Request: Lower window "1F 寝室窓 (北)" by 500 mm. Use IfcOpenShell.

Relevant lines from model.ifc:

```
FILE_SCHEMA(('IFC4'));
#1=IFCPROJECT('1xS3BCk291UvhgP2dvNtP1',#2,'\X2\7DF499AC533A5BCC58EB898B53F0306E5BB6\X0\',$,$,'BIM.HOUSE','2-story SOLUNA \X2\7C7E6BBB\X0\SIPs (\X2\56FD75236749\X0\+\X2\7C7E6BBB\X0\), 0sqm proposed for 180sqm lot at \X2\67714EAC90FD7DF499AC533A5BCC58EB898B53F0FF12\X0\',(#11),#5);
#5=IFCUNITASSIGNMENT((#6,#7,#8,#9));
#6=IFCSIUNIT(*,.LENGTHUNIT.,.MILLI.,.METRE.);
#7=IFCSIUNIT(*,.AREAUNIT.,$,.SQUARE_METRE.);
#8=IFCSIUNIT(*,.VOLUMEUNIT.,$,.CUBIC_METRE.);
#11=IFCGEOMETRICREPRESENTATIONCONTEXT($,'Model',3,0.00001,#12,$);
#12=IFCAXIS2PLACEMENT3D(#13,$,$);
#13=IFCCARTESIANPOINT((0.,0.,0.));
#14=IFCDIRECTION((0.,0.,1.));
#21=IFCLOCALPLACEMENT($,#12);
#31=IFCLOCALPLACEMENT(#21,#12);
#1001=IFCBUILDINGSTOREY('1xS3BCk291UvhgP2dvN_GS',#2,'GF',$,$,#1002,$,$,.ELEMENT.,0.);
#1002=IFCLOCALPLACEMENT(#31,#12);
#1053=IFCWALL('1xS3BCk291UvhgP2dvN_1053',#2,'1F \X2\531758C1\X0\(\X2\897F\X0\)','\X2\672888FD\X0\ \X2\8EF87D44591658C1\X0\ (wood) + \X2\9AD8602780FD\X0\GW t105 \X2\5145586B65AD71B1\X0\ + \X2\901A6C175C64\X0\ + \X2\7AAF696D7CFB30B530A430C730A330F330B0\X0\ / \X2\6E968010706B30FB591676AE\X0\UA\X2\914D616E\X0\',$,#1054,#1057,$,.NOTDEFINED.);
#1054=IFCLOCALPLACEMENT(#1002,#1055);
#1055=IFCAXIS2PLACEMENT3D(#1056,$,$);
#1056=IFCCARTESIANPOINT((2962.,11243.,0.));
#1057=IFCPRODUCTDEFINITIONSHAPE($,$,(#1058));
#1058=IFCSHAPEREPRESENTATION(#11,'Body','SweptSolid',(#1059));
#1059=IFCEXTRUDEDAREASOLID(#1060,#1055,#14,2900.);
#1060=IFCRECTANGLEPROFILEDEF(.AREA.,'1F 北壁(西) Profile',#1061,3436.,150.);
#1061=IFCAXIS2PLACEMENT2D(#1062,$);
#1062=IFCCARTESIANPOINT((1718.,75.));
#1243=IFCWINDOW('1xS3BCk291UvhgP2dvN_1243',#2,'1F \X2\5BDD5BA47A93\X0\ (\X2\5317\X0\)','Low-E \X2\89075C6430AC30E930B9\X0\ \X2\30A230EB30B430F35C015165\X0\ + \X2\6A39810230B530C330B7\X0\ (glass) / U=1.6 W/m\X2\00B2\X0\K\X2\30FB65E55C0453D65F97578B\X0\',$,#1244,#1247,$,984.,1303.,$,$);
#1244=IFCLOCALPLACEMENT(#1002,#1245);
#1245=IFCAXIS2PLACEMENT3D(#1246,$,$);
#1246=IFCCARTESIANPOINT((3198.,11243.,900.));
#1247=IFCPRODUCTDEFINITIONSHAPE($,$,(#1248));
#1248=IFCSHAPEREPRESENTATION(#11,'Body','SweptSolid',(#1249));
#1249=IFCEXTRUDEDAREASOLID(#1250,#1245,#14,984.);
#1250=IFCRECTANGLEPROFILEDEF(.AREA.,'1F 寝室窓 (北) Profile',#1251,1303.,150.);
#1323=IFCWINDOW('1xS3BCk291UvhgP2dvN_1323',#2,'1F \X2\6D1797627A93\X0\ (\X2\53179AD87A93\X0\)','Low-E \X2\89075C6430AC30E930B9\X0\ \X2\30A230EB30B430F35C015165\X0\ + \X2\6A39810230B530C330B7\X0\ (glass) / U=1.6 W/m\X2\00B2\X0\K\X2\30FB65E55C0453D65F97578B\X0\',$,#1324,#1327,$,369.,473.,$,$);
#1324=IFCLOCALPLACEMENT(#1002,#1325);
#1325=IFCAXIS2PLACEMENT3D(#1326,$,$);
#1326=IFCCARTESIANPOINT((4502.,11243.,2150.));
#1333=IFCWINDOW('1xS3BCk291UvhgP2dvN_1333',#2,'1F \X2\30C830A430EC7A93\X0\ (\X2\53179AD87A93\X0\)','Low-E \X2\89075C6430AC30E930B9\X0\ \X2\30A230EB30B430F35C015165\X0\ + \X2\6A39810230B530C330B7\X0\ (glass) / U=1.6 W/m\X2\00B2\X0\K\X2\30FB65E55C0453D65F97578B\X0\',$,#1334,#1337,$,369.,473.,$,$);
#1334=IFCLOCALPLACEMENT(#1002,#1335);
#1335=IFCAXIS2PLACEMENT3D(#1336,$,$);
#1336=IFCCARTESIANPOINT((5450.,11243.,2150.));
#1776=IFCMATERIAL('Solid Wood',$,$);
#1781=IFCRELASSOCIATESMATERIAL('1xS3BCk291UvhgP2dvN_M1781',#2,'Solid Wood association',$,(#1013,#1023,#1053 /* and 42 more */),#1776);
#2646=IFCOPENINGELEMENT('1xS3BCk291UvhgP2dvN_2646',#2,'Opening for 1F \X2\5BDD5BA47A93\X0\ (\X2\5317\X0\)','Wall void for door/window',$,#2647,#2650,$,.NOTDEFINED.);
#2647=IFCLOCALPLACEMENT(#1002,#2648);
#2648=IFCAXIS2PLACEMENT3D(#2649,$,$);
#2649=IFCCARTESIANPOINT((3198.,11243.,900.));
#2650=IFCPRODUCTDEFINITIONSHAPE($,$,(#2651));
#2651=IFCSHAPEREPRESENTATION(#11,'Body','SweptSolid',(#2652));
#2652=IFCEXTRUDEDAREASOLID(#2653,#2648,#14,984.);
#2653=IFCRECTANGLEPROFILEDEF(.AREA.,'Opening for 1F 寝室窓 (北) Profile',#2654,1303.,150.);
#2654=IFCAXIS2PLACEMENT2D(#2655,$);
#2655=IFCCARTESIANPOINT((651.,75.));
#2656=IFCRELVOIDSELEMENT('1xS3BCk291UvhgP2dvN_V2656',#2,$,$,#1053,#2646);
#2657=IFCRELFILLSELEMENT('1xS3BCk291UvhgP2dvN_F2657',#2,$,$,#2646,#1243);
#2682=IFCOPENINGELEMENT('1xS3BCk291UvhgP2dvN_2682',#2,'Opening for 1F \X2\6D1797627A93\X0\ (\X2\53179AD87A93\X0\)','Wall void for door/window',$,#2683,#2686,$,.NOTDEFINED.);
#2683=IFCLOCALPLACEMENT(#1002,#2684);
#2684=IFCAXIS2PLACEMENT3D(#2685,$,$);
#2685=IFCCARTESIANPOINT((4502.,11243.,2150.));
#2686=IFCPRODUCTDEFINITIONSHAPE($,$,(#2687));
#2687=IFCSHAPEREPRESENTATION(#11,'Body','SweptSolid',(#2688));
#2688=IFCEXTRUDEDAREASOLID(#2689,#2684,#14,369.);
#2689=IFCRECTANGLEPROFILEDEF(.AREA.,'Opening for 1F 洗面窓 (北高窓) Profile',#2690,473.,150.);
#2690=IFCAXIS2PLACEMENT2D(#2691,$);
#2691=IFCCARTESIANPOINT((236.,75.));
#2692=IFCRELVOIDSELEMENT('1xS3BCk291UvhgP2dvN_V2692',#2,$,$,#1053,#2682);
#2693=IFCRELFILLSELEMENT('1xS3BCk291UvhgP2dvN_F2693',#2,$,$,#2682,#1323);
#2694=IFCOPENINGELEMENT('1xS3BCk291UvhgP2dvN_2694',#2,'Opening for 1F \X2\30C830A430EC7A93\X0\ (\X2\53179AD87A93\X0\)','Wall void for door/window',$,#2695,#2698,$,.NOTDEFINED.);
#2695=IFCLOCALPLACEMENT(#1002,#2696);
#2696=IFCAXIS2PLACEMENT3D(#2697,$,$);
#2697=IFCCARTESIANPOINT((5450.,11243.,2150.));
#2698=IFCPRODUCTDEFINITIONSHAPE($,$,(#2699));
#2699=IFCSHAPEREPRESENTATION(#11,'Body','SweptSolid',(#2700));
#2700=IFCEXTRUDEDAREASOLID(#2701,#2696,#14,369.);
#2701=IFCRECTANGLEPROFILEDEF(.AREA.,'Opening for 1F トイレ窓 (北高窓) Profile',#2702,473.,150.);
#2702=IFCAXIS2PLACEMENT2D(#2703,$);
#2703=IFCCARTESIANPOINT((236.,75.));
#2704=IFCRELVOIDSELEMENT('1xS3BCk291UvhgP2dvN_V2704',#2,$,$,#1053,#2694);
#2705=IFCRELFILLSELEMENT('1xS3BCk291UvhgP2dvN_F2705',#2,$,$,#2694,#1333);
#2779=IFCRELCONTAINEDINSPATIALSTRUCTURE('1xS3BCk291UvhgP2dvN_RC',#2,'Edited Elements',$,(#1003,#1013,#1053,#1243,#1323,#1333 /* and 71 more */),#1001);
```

```python
import numpy as np
import ifcopenshell
import ifcopenshell.api.geometry
import ifcopenshell.util.placement
import ifcopenshell.util.unit

model = ifcopenshell.open("model.ifc")
unit_scale = ifcopenshell.util.unit.calculate_unit_scale(model)

window = model.by_guid("1xS3BCk291UvhgP2dvN_1243")
opening = window.FillsVoids[0].RelatingOpeningElement
dz = -500.0

shift = np.array([0.0, 0.0, dz])
# The window is not placed relative to its opening, so move both.
for product in (opening, window):
    matrix = ifcopenshell.util.placement.get_local_placement(product.ObjectPlacement)
    matrix[:3, 3] += shift
    ifcopenshell.api.geometry.edit_object_placement(model, product=product, matrix=matrix, is_si=False)

print(f"moved by {dz * unit_scale:+.3f} m")

model.write("model_edited.ifc")
```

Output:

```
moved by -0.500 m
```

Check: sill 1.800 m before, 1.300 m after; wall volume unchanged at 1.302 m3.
